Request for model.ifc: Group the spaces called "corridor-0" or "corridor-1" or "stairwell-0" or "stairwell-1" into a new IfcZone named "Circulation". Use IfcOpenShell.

First a look at what the model holds.

```python
import ifcopenshell

model = ifcopenshell.open("model.ifc")
print(model.schema)
seen = {}
for space in model.by_type("IfcSpace"):
    seen[space.Name] = seen.get(space.Name, 0) + 1
for name, count in sorted(seen.items(), key=str):
    print(count, "x", name)
print("zones:", [z.Name for z in model.by_type("IfcZone")][:20])
```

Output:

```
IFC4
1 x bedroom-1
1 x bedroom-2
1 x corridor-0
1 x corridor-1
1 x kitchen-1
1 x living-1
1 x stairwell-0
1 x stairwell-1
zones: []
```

```python
import ifcopenshell
import ifcopenshell.api.group
import ifcopenshell.api.root

model = ifcopenshell.open("model.ifc")

names = {"corridor-0", "corridor-1", "stairwell-0", "stairwell-1"}
spaces = [s for s in model.by_type("IfcSpace") if s.Name in names]

zone = ifcopenshell.api.root.create_entity(model, ifc_class="IfcZone", name="Circulation")
ifcopenshell.api.group.assign_group(model, products=spaces, group=zone)
print(len(spaces), "spaces in", zone.Name)

model.write("model_updated.ifc")
```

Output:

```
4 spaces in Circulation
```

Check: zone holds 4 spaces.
